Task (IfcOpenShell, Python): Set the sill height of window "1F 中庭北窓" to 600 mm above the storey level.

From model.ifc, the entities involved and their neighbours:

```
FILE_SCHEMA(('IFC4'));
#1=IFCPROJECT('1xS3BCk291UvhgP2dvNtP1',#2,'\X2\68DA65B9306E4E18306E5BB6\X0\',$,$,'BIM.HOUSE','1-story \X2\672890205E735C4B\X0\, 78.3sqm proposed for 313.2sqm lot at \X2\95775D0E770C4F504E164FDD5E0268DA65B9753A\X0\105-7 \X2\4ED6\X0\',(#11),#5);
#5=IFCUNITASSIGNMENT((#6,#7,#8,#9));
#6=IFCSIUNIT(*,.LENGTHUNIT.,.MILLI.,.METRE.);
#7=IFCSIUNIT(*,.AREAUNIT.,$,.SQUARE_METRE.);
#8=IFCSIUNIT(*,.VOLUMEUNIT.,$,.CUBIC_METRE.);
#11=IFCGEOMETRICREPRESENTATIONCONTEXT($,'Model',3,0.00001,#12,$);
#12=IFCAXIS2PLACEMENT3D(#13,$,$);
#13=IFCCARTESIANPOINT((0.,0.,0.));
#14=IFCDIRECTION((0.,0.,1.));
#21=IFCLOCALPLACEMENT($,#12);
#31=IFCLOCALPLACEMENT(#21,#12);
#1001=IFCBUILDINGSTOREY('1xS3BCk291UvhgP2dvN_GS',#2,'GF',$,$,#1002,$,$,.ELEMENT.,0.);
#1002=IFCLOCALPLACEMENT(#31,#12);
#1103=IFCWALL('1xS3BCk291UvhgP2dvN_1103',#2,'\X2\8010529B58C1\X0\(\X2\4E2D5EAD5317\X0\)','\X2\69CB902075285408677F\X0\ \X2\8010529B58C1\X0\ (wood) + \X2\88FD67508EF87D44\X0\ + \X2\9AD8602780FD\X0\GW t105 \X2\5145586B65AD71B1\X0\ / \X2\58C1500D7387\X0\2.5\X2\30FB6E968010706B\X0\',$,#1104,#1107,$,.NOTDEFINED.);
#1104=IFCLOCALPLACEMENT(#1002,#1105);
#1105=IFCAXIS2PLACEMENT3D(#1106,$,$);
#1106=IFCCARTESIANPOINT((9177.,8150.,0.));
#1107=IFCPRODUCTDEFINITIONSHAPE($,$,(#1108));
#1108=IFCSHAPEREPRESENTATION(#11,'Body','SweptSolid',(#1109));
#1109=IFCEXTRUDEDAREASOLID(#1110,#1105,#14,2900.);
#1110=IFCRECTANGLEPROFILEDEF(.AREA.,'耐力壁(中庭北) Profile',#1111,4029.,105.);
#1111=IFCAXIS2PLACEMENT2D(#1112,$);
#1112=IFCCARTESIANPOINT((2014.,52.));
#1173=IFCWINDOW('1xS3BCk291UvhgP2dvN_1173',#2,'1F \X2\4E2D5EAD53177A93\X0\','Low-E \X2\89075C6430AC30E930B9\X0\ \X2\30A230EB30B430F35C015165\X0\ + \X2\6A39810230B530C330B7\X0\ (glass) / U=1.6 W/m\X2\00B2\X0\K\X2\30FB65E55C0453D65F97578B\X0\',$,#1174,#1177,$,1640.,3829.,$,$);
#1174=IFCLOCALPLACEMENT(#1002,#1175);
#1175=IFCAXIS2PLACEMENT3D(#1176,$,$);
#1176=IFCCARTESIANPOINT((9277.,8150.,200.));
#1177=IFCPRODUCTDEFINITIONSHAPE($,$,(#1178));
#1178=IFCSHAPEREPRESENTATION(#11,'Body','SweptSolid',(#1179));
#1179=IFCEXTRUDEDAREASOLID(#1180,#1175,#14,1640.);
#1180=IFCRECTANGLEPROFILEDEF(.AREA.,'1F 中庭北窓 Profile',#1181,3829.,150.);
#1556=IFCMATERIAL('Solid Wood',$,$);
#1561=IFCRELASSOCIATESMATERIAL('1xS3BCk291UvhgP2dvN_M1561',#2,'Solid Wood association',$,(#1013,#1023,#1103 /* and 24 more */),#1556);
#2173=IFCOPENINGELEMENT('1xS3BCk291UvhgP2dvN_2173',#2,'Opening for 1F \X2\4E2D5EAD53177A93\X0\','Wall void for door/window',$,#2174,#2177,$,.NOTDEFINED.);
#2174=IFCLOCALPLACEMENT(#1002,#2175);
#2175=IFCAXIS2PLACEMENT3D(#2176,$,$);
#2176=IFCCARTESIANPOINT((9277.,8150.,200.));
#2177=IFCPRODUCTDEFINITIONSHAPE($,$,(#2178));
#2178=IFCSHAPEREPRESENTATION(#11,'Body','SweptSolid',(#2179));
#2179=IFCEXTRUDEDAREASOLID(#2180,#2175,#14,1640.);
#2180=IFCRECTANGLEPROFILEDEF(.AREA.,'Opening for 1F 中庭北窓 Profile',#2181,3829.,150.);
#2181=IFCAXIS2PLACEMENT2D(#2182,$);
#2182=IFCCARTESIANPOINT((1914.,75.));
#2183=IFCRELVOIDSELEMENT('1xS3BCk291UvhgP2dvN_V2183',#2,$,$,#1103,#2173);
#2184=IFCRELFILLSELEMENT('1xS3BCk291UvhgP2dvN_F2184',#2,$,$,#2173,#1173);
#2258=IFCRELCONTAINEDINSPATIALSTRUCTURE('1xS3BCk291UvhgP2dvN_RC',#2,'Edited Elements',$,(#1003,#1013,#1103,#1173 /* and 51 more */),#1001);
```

```python
import numpy as np
import ifcopenshell
import ifcopenshell.api.geometry
import ifcopenshell.geom
import ifcopenshell.util.element
import ifcopenshell.util.placement
import ifcopenshell.util.shape
import ifcopenshell.util.unit

model = ifcopenshell.open("model.ifc")
unit_scale = ifcopenshell.util.unit.calculate_unit_scale(model)

window = model.by_id(1173)
opening = window.FillsVoids[0].RelatingOpeningElement
storey = ifcopenshell.util.element.get_container(window, ifc_class="IfcBuildingStorey")
level = ifcopenshell.util.placement.get_local_placement(storey.ObjectPlacement)[2, 3]

# The opening's origin need not be at the sill, so measure its lowest point.
shape = ifcopenshell.geom.create_shape(ifcopenshell.geom.settings(), opening)
bottom = ifcopenshell.util.shape.get_shape_bottom_elevation(shape, shape.geometry) / unit_scale
dz = level + 600.0 - bottom

shift = np.array([0.0, 0.0, dz])
# The window is not placed relative to its opening, so move both.
for product in (opening, window):
    matrix = ifcopenshell.util.placement.get_local_placement(product.ObjectPlacement)
    matrix[:3, 3] += shift
    ifcopenshell.api.geometry.edit_object_placement(model, product=product, matrix=matrix, is_si=False)

print(f"moved by {dz * unit_scale:+.3f} m")

model.write("model_updated.ifc")
```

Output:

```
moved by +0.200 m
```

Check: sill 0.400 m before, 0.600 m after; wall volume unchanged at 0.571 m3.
